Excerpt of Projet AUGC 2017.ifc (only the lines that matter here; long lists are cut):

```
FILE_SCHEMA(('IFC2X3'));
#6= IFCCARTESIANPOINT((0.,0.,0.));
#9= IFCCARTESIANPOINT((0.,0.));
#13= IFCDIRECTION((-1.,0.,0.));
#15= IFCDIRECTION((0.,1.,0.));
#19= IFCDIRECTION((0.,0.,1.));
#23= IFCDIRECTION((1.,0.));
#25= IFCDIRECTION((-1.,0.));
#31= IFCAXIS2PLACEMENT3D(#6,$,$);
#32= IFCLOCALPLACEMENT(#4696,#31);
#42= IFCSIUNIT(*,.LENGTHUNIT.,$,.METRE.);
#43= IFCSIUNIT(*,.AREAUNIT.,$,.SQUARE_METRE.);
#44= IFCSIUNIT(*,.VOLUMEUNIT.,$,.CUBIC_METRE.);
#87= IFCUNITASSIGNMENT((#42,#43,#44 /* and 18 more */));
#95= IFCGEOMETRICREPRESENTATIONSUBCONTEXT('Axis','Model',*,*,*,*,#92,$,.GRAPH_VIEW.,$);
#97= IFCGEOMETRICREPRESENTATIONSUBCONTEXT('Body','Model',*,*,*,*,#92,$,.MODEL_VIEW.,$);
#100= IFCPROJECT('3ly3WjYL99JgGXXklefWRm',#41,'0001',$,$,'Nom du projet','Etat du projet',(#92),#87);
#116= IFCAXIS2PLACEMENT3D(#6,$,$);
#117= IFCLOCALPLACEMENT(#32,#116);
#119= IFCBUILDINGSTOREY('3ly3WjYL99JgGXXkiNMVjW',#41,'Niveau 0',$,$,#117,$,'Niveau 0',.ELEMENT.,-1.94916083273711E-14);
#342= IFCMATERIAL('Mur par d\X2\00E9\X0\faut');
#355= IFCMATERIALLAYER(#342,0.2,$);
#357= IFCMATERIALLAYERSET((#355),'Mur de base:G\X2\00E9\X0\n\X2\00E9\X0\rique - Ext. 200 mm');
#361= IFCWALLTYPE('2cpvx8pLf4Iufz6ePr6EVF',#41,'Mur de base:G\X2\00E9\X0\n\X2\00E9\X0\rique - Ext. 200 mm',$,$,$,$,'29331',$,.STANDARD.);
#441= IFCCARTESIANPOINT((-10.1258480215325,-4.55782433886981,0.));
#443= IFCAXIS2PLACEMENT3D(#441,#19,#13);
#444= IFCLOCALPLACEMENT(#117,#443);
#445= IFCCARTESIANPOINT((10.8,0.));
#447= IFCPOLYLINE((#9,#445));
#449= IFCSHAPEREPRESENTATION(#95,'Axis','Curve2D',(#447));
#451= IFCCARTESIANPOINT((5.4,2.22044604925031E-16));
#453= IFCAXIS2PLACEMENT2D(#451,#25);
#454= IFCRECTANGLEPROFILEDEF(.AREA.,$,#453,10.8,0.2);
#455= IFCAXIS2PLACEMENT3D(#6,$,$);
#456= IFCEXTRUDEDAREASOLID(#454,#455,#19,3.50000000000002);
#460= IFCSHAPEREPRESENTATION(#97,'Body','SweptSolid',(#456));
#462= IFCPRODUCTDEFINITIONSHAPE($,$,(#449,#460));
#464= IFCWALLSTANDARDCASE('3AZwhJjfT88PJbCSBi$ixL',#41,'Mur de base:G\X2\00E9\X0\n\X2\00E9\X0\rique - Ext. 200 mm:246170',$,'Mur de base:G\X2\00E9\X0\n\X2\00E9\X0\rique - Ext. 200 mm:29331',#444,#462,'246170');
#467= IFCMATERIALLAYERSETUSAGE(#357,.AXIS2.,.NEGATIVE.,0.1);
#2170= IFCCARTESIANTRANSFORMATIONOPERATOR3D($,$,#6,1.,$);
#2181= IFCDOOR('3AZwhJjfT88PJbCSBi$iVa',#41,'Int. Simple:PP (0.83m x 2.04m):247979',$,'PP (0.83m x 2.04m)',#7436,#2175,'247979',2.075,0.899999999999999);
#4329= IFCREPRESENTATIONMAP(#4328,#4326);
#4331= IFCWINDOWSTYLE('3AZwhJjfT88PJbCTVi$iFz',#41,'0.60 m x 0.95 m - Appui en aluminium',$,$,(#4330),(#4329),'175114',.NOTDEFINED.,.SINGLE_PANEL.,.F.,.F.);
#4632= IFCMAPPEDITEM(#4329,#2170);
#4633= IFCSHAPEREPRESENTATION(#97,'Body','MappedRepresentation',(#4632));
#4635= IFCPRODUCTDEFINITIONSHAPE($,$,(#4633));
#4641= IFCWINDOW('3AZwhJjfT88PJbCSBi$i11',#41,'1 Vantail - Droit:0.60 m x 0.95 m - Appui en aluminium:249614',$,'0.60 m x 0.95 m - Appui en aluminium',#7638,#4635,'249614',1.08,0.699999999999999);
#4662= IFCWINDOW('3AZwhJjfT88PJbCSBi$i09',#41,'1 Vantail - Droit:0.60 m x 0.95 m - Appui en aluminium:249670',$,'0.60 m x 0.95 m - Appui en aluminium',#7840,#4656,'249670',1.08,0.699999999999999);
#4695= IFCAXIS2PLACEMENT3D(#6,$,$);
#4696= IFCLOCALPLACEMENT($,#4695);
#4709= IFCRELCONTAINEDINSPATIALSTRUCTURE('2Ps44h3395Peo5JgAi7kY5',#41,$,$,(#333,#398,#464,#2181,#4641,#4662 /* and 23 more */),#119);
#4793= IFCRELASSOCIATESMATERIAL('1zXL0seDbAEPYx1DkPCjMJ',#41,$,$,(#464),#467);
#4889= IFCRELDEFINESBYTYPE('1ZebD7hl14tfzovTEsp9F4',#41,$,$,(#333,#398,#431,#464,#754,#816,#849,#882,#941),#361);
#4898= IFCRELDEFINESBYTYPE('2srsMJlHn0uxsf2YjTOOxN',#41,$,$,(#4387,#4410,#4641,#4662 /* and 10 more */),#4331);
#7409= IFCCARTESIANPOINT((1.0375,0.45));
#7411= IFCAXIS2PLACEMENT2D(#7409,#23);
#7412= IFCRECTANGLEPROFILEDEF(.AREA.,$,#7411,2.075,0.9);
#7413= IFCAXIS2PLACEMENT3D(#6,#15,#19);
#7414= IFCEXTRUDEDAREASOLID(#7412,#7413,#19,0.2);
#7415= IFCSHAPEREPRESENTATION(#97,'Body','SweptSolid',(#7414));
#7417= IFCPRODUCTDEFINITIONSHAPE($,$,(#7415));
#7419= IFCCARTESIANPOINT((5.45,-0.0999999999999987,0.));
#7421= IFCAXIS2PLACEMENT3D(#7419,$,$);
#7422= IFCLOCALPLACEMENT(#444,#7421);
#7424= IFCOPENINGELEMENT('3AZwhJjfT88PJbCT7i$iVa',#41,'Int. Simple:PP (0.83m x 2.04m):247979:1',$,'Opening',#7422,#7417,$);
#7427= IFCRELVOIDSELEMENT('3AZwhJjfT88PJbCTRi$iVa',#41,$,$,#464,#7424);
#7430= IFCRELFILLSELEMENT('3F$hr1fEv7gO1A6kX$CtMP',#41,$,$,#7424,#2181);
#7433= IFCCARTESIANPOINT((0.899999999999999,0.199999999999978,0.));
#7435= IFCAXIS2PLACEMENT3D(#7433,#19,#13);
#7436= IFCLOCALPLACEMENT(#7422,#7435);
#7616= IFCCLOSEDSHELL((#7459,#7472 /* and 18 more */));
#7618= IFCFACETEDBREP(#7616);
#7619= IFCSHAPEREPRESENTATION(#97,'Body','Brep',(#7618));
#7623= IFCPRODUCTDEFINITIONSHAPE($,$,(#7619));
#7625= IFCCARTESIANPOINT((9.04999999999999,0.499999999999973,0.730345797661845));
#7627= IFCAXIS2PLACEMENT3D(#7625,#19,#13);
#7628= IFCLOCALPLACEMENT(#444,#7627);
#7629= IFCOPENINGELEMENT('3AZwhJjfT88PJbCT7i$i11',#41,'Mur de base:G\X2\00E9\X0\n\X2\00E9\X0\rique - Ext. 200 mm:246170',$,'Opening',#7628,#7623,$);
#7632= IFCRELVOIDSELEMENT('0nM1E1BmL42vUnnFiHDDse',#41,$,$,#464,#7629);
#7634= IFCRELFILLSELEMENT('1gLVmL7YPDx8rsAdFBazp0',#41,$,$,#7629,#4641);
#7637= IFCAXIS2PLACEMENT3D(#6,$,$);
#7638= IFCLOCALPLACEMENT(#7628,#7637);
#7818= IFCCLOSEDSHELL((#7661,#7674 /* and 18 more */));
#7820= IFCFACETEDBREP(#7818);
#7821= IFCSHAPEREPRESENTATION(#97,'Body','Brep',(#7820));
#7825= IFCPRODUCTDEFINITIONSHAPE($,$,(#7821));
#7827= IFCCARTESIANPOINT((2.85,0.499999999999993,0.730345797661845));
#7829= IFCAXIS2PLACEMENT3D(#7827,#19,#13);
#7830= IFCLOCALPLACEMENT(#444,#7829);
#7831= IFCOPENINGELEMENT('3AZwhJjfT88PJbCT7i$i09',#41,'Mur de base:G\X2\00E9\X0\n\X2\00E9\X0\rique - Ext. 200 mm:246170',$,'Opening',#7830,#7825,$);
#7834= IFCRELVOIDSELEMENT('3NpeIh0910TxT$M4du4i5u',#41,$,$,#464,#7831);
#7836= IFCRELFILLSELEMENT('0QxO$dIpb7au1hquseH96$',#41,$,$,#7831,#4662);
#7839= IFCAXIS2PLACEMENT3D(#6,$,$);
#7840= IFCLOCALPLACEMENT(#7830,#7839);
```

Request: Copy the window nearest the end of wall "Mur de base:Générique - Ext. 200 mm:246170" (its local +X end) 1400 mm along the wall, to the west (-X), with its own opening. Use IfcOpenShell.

```python
import ifcopenshell
import ifcopenshell.api.feature
import ifcopenshell.api.geometry
import ifcopenshell.api.root
import ifcopenshell.geom
import ifcopenshell.util.element
import ifcopenshell.util.placement
import ifcopenshell.util.shape

model = ifcopenshell.open("Projet AUGC 2017.ifc")
settings = ifcopenshell.geom.settings()


def volume(element):
    """Net volume in cubic metres, openings subtracted."""
    shape = ifcopenshell.geom.create_shape(settings, element)
    return ifcopenshell.util.shape.get_volume(shape.geometry)


def reuse_history(source, copy):
    """copy_class also copies each property set's owner history, people and application; keep the originals."""
    for rel in copy.IsDefinedBy:
        if rel.is_a("IfcRelDefinesByProperties") and (history := rel.RelatingPropertyDefinition.OwnerHistory):
            rel.RelatingPropertyDefinition.OwnerHistory = source.OwnerHistory
            ifcopenshell.util.element.remove_deep2(model, history)


window = model.by_guid("3AZwhJjfT88PJbCSBi$i11")
opening = window.FillsVoids[0].RelatingOpeningElement
wall = opening.VoidsElements[0].RelatingBuildingElement
before = volume(wall)
shift = ifcopenshell.util.placement.get_local_placement(wall.ObjectPlacement)[:3, 0] * 1.4

# copy_class copies the void relationship, type, container and properties, but no geometry.
new_opening = ifcopenshell.api.root.copy_class(model, product=opening)
new_opening.Representation = ifcopenshell.util.element.copy_deep(
    model, opening.Representation, exclude=["IfcGeometricRepresentationContext", "IfcRepresentationMap"]
)
new_opening.Name = "Mur de base:Générique - Ext. 200 mm"
new_window = ifcopenshell.api.root.copy_class(model, product=window)
new_window.Representation = ifcopenshell.util.element.copy_deep(
    model, window.Representation, exclude=["IfcGeometricRepresentationContext", "IfcRepresentationMap"]
)
new_window.Name = "1 Vantail - Droit:0.60 m x 0.95 m - Appui en aluminium"
new_window.Tag = None
reuse_history(window, new_window)
fills = ifcopenshell.api.feature.add_filling(model, opening=new_opening, element=new_window)
fills.OwnerHistory = new_window.OwnerHistory  # required in IFC2X3

for old, new in ((opening, new_opening), (window, new_window)):
    matrix = ifcopenshell.util.placement.get_local_placement(old.ObjectPlacement)
    matrix[:3, 3] += shift
    ifcopenshell.api.geometry.edit_object_placement(model, product=new, matrix=matrix, is_si=False)

after = volume(wall)

print(f"wall volume {before:.3f} -> {after:.3f} m3")

model.write("Projet AUGC 2017_edited.ifc")
```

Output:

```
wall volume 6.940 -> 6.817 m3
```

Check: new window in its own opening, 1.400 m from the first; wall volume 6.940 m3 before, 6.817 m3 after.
